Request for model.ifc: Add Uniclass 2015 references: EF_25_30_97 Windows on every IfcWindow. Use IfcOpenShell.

First a look at what the model holds.

```python
import ifcopenshell

model = ifcopenshell.open("model.ifc")
print(model.schema)
print("classifications:", [c.Name for c in model.by_type("IfcClassification")])
for ifc_class in ("IfcDoor", "IfcRoof", "IfcStair", "IfcWall", "IfcWindow"):
    print(ifc_class, len(model.by_type(ifc_class)))
```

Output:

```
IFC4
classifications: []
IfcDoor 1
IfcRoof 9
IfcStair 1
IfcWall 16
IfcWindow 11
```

```python
import ifcopenshell
import ifcopenshell.api.classification

model = ifcopenshell.open("model.ifc")

system = ifcopenshell.api.classification.add_classification(model, classification="Uniclass 2015")

codes = {
    "IfcWindow": ("EF_25_30_97", "Windows"),
}
for ifc_class, (code, name) in codes.items():
    products = model.by_type(ifc_class)
    ifcopenshell.api.classification.add_reference(
        model, products=products, classification=system, identification=code, name=name
    )
    print(code, len(products))

model.write("model_edited.ifc")
```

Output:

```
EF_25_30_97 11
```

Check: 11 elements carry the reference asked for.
